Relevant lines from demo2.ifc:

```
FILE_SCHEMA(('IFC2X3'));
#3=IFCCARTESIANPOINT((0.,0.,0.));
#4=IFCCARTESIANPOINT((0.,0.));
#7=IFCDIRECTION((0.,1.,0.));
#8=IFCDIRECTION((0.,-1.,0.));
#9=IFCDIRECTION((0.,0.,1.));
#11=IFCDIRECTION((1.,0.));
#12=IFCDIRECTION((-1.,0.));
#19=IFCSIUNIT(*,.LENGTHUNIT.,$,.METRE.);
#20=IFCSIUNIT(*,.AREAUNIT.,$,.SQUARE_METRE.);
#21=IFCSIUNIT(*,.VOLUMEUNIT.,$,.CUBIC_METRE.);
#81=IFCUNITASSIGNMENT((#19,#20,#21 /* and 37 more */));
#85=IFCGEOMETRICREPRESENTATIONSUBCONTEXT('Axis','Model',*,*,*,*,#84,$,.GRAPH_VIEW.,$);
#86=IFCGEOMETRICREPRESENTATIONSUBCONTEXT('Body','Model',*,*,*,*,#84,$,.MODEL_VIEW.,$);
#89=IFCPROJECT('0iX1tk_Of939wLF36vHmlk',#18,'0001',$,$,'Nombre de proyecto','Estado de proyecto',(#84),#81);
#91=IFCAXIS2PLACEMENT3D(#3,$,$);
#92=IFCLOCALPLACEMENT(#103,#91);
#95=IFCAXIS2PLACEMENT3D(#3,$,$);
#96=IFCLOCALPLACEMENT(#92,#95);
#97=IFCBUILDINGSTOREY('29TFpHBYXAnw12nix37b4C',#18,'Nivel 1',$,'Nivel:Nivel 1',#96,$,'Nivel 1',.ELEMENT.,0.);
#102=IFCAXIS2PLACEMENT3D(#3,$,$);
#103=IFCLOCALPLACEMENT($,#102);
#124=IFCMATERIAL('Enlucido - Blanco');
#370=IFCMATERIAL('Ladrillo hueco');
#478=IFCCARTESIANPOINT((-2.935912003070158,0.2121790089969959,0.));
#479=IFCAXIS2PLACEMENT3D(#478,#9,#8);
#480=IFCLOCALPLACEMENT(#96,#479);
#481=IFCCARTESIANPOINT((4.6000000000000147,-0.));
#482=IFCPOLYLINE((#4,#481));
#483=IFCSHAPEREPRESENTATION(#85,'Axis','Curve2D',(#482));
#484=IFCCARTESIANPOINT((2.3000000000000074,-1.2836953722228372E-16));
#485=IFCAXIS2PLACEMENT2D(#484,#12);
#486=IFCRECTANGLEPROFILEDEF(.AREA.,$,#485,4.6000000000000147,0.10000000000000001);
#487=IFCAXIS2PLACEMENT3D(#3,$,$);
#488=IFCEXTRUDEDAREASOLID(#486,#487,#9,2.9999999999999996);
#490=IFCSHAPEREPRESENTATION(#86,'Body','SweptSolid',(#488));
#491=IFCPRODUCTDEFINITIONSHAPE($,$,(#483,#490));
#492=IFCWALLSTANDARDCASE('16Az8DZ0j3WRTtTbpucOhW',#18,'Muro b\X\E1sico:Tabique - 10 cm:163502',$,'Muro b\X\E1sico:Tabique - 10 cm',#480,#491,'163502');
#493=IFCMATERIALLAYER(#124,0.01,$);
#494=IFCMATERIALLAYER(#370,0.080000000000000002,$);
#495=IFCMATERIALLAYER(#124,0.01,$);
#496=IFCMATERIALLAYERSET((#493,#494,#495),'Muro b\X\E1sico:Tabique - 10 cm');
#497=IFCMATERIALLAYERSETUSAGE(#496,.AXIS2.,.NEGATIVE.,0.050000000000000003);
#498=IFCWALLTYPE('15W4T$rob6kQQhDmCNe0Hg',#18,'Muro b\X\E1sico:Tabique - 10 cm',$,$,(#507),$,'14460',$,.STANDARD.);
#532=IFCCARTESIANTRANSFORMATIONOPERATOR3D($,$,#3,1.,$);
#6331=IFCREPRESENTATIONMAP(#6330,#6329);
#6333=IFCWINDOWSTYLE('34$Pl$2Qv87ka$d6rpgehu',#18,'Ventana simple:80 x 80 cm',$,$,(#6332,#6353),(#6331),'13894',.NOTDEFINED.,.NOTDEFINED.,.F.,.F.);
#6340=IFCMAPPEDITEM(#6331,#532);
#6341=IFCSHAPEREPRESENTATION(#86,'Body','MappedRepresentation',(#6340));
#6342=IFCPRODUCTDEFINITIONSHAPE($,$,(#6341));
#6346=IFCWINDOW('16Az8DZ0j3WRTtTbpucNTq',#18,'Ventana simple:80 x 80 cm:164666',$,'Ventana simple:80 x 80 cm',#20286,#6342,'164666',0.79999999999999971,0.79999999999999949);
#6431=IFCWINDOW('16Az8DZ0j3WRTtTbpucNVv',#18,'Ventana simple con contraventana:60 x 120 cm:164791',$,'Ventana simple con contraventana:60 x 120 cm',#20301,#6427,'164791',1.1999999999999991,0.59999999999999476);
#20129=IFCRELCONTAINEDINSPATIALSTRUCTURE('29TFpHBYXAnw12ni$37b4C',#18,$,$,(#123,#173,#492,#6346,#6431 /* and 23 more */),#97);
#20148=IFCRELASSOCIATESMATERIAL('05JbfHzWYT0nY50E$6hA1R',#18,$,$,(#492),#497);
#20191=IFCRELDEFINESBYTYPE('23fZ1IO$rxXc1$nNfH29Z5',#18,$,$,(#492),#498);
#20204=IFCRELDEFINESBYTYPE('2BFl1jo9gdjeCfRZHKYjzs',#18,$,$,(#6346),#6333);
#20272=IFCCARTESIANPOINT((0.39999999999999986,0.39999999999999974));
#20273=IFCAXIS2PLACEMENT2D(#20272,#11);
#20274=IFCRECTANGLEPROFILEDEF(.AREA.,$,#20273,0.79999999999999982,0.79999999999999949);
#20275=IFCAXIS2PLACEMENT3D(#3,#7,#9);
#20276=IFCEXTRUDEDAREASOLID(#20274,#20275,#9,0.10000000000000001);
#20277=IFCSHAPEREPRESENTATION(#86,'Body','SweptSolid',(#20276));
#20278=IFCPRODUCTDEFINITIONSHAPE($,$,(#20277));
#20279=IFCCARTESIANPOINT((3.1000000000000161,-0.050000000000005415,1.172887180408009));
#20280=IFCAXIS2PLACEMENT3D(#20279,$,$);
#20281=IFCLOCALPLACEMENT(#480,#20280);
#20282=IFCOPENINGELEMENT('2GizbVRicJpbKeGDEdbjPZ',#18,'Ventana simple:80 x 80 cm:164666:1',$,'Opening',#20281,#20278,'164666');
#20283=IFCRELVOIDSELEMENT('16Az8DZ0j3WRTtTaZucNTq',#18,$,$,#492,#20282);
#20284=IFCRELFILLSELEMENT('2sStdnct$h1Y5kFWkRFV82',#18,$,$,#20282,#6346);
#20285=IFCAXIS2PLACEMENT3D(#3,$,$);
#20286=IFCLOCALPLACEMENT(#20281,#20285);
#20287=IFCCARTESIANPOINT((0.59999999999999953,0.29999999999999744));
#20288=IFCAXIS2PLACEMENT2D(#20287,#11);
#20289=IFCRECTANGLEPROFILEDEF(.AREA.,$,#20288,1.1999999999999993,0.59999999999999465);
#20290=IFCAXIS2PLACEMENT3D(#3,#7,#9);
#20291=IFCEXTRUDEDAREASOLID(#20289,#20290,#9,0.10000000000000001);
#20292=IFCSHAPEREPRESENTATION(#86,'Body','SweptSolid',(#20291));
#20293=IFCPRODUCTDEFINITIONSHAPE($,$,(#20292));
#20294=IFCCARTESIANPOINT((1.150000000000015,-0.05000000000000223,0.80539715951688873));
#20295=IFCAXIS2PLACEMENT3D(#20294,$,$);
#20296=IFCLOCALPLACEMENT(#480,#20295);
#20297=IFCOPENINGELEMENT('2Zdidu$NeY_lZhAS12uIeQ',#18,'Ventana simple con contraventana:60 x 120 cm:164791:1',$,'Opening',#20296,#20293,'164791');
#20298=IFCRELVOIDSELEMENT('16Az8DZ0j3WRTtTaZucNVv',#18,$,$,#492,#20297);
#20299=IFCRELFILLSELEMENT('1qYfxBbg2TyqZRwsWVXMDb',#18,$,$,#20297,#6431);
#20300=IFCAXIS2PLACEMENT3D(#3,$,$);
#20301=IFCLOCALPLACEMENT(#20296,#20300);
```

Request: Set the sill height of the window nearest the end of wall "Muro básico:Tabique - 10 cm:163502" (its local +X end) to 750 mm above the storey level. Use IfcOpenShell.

```python
import numpy as np
import ifcopenshell
import ifcopenshell.api.geometry
import ifcopenshell.geom
import ifcopenshell.util.element
import ifcopenshell.util.placement
import ifcopenshell.util.shape
import ifcopenshell.util.unit

model = ifcopenshell.open("demo2.ifc")
unit_scale = ifcopenshell.util.unit.calculate_unit_scale(model)

window = model.by_guid("16Az8DZ0j3WRTtTbpucNTq")
opening = window.FillsVoids[0].RelatingOpeningElement
storey = ifcopenshell.util.element.get_container(window, ifc_class="IfcBuildingStorey")
level = ifcopenshell.util.placement.get_local_placement(storey.ObjectPlacement)[2, 3]

# The opening's origin need not be at the sill, so measure its lowest point.
shape = ifcopenshell.geom.create_shape(ifcopenshell.geom.settings(), opening)
bottom = ifcopenshell.util.shape.get_shape_bottom_elevation(shape, shape.geometry) / unit_scale
dz = level + 0.75 / unit_scale - bottom

shift = np.array([0.0, 0.0, dz])
# The window is placed relative to its opening, so it follows when the opening moves.
matrix = ifcopenshell.util.placement.get_local_placement(opening.ObjectPlacement)
matrix[:3, 3] += shift
ifcopenshell.api.geometry.edit_object_placement(
    model, product=opening, matrix=matrix, is_si=False, should_transform_children=True
)

print(f"moved by {dz * unit_scale:+.3f} m")

model.write("demo2_edited.ifc")
```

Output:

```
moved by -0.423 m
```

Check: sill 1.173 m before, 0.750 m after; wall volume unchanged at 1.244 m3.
